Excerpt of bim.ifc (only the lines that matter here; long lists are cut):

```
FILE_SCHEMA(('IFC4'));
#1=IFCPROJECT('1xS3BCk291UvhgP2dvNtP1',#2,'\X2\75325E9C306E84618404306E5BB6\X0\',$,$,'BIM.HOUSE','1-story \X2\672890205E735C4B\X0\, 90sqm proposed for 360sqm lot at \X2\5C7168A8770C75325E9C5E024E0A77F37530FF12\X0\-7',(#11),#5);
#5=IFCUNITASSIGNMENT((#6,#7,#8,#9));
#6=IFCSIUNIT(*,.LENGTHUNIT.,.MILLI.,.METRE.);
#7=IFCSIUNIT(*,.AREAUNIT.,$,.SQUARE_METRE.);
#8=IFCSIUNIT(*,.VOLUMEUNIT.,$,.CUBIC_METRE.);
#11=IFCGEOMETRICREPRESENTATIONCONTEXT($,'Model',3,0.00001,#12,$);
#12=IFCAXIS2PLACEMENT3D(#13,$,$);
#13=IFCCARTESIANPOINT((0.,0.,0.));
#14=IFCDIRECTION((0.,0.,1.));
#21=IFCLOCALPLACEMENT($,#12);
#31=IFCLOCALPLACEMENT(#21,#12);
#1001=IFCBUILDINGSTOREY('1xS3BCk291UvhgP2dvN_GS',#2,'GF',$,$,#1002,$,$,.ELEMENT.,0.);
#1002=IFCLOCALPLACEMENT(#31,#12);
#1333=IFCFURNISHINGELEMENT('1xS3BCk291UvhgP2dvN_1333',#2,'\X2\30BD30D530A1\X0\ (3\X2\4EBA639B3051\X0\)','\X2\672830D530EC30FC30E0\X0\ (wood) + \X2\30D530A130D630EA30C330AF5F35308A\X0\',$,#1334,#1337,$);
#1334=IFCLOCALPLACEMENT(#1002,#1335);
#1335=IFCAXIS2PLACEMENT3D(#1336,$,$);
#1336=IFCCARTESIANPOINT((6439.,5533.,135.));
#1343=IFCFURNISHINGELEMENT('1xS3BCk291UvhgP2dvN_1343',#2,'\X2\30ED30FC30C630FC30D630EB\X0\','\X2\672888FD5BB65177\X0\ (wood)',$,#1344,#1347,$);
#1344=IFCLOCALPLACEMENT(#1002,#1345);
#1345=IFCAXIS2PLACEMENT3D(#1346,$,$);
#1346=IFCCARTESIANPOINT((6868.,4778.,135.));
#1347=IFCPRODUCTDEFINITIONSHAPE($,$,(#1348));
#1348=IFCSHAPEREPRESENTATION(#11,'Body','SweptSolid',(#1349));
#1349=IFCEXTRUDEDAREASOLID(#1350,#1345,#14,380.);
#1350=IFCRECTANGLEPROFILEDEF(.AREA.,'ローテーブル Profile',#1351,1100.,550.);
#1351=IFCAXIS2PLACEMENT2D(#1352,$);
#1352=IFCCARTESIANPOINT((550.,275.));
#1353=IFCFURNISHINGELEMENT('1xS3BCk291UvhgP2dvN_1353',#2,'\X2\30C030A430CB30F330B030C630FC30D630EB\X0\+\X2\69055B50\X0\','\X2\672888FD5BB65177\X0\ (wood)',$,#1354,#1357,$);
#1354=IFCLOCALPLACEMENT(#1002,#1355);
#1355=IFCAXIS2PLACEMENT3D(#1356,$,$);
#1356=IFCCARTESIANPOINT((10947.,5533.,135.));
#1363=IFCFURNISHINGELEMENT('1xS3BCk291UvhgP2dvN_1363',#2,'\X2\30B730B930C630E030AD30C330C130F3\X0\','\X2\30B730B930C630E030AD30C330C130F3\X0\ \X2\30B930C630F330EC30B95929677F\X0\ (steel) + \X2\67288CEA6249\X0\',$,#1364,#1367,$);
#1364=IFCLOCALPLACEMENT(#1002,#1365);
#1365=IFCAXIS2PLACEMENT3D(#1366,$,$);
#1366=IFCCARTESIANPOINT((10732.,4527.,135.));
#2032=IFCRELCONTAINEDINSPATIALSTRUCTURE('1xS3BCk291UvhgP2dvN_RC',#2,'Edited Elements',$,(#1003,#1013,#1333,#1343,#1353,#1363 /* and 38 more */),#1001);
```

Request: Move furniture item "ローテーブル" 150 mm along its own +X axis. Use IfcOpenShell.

```python
import ifcopenshell
import ifcopenshell.api.geometry
import ifcopenshell.util.placement

model = ifcopenshell.open("bim.ifc")

item = model.by_guid("1xS3BCk291UvhgP2dvN_1343")
matrix = ifcopenshell.util.placement.get_local_placement(item.ObjectPlacement)
matrix[:3, 3] += matrix[:3, 0] * 150.0
ifcopenshell.api.geometry.edit_object_placement(model, product=item, matrix=matrix, is_si=False)

print(ifcopenshell.util.placement.get_local_placement(item.ObjectPlacement).round(3) + 0.0)

model.write("bim_updated.ifc")
```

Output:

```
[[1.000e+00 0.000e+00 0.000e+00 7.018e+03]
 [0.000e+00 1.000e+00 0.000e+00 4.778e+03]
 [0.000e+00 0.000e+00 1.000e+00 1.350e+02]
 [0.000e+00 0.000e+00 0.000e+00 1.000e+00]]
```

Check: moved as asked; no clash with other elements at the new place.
